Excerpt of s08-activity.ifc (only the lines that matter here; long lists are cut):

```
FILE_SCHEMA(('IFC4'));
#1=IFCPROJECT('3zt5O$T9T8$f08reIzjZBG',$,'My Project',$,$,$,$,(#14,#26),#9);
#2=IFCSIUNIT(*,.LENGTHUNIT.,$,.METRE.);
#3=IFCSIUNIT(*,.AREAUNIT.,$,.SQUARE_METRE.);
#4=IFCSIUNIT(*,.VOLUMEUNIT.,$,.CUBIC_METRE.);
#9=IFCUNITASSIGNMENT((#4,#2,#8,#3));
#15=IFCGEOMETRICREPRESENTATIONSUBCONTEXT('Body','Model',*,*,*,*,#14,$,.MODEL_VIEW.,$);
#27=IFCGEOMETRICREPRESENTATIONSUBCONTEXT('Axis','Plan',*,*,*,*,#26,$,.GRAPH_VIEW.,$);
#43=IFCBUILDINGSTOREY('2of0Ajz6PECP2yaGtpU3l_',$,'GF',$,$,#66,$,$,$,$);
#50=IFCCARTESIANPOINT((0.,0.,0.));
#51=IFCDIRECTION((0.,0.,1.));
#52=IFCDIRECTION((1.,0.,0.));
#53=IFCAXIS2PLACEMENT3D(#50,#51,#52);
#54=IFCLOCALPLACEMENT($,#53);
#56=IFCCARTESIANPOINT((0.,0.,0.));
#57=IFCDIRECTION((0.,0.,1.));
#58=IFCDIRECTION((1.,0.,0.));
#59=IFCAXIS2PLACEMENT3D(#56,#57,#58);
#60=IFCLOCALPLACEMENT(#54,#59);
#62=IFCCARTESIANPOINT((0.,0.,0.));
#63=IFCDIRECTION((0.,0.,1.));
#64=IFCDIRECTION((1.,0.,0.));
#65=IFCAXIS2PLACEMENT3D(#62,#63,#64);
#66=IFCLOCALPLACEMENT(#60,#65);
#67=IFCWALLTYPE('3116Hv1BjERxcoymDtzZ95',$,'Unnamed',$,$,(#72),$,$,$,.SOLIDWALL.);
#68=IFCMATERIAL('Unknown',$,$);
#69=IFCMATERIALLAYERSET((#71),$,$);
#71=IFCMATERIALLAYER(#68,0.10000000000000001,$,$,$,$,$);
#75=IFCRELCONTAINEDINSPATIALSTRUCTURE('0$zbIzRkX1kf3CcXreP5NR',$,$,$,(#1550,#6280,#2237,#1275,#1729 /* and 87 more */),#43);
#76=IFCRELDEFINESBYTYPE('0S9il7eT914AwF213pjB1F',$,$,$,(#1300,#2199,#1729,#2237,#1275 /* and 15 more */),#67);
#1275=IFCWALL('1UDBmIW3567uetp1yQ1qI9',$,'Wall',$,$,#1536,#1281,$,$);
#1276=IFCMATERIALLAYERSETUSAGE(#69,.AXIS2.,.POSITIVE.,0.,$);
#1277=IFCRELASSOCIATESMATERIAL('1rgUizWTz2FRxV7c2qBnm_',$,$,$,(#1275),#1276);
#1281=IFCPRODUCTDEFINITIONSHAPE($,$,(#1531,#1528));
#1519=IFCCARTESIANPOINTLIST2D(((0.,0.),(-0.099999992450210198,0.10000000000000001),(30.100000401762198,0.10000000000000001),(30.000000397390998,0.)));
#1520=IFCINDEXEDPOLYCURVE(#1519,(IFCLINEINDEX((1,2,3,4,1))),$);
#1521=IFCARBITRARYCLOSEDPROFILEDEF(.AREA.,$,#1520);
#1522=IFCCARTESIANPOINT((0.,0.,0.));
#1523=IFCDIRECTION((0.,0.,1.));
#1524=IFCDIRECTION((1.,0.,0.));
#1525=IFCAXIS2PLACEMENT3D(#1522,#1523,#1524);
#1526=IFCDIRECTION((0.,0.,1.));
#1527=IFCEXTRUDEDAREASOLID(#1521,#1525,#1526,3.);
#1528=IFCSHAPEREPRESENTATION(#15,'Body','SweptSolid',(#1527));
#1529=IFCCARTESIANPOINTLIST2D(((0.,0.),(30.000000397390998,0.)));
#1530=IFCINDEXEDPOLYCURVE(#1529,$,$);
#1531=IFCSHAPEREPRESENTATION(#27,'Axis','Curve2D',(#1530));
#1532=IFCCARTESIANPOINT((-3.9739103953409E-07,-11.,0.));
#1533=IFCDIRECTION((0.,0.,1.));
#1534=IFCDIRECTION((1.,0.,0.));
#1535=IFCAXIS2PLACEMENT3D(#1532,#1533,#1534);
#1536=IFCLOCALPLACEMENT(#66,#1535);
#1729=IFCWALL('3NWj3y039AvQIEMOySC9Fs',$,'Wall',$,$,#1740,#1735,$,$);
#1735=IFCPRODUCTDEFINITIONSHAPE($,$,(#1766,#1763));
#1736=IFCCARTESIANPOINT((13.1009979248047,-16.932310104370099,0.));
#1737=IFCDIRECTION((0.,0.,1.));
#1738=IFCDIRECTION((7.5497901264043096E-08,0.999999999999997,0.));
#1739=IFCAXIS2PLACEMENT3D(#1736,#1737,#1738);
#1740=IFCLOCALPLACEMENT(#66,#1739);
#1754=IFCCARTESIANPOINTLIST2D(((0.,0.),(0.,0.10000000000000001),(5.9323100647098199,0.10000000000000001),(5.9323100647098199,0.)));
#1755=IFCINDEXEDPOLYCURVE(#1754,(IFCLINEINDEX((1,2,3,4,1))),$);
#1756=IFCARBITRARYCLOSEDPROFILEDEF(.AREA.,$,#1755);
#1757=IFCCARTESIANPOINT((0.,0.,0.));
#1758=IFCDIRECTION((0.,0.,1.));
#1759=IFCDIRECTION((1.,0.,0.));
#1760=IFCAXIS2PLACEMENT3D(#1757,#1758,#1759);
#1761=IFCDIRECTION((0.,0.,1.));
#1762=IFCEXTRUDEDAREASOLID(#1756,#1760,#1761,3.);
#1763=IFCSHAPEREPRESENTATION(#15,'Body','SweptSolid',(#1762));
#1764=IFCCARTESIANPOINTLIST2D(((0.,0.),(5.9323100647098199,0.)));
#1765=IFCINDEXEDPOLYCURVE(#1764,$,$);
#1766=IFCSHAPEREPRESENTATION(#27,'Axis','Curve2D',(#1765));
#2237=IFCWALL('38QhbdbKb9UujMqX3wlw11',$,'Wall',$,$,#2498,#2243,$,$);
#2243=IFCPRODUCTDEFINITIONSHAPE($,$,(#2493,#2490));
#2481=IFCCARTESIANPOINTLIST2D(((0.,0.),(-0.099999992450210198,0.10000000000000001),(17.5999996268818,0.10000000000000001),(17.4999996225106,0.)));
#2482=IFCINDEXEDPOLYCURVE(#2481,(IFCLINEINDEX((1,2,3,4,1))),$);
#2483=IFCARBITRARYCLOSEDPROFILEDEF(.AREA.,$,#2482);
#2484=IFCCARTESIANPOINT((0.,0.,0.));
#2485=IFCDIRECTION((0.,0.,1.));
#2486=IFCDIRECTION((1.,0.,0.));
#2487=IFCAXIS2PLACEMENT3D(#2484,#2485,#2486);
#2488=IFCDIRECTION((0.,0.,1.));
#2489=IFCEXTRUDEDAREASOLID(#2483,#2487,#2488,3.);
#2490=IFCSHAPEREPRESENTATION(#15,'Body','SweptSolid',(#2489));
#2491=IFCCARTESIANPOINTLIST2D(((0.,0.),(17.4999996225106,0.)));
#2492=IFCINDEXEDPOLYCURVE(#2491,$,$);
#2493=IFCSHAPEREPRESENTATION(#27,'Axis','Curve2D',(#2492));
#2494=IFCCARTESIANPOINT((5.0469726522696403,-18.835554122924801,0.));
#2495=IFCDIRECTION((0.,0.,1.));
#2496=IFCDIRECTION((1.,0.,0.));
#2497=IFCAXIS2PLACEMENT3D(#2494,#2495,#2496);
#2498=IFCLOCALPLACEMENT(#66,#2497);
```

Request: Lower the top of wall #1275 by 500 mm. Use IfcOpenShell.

```python
import ifcopenshell
import ifcopenshell.geom
import ifcopenshell.util.representation
import ifcopenshell.util.shape

model = ifcopenshell.open("s08-activity.ifc")
settings = ifcopenshell.geom.settings()


def volume(element):
    """Net volume in cubic metres, openings subtracted."""
    shape = ifcopenshell.geom.create_shape(settings, element)
    return ifcopenshell.util.shape.get_volume(shape.geometry)


wall = model.by_guid("1UDBmIW3567uetp1yQ1qI9")
before = volume(wall)

body = ifcopenshell.util.representation.get_representation(wall, "Model", "Body")
solid = body.Items[0]
old_height = solid.Depth
solid.Depth -= 0.5
after = volume(wall)

print(f"height {old_height:g} -> {solid.Depth:g}, volume {before:.3f} -> {after:.3f} m3")

model.write("s08-activity_rev.ifc")
```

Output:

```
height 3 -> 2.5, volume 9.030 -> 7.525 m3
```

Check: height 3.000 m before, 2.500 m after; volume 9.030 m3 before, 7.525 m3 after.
